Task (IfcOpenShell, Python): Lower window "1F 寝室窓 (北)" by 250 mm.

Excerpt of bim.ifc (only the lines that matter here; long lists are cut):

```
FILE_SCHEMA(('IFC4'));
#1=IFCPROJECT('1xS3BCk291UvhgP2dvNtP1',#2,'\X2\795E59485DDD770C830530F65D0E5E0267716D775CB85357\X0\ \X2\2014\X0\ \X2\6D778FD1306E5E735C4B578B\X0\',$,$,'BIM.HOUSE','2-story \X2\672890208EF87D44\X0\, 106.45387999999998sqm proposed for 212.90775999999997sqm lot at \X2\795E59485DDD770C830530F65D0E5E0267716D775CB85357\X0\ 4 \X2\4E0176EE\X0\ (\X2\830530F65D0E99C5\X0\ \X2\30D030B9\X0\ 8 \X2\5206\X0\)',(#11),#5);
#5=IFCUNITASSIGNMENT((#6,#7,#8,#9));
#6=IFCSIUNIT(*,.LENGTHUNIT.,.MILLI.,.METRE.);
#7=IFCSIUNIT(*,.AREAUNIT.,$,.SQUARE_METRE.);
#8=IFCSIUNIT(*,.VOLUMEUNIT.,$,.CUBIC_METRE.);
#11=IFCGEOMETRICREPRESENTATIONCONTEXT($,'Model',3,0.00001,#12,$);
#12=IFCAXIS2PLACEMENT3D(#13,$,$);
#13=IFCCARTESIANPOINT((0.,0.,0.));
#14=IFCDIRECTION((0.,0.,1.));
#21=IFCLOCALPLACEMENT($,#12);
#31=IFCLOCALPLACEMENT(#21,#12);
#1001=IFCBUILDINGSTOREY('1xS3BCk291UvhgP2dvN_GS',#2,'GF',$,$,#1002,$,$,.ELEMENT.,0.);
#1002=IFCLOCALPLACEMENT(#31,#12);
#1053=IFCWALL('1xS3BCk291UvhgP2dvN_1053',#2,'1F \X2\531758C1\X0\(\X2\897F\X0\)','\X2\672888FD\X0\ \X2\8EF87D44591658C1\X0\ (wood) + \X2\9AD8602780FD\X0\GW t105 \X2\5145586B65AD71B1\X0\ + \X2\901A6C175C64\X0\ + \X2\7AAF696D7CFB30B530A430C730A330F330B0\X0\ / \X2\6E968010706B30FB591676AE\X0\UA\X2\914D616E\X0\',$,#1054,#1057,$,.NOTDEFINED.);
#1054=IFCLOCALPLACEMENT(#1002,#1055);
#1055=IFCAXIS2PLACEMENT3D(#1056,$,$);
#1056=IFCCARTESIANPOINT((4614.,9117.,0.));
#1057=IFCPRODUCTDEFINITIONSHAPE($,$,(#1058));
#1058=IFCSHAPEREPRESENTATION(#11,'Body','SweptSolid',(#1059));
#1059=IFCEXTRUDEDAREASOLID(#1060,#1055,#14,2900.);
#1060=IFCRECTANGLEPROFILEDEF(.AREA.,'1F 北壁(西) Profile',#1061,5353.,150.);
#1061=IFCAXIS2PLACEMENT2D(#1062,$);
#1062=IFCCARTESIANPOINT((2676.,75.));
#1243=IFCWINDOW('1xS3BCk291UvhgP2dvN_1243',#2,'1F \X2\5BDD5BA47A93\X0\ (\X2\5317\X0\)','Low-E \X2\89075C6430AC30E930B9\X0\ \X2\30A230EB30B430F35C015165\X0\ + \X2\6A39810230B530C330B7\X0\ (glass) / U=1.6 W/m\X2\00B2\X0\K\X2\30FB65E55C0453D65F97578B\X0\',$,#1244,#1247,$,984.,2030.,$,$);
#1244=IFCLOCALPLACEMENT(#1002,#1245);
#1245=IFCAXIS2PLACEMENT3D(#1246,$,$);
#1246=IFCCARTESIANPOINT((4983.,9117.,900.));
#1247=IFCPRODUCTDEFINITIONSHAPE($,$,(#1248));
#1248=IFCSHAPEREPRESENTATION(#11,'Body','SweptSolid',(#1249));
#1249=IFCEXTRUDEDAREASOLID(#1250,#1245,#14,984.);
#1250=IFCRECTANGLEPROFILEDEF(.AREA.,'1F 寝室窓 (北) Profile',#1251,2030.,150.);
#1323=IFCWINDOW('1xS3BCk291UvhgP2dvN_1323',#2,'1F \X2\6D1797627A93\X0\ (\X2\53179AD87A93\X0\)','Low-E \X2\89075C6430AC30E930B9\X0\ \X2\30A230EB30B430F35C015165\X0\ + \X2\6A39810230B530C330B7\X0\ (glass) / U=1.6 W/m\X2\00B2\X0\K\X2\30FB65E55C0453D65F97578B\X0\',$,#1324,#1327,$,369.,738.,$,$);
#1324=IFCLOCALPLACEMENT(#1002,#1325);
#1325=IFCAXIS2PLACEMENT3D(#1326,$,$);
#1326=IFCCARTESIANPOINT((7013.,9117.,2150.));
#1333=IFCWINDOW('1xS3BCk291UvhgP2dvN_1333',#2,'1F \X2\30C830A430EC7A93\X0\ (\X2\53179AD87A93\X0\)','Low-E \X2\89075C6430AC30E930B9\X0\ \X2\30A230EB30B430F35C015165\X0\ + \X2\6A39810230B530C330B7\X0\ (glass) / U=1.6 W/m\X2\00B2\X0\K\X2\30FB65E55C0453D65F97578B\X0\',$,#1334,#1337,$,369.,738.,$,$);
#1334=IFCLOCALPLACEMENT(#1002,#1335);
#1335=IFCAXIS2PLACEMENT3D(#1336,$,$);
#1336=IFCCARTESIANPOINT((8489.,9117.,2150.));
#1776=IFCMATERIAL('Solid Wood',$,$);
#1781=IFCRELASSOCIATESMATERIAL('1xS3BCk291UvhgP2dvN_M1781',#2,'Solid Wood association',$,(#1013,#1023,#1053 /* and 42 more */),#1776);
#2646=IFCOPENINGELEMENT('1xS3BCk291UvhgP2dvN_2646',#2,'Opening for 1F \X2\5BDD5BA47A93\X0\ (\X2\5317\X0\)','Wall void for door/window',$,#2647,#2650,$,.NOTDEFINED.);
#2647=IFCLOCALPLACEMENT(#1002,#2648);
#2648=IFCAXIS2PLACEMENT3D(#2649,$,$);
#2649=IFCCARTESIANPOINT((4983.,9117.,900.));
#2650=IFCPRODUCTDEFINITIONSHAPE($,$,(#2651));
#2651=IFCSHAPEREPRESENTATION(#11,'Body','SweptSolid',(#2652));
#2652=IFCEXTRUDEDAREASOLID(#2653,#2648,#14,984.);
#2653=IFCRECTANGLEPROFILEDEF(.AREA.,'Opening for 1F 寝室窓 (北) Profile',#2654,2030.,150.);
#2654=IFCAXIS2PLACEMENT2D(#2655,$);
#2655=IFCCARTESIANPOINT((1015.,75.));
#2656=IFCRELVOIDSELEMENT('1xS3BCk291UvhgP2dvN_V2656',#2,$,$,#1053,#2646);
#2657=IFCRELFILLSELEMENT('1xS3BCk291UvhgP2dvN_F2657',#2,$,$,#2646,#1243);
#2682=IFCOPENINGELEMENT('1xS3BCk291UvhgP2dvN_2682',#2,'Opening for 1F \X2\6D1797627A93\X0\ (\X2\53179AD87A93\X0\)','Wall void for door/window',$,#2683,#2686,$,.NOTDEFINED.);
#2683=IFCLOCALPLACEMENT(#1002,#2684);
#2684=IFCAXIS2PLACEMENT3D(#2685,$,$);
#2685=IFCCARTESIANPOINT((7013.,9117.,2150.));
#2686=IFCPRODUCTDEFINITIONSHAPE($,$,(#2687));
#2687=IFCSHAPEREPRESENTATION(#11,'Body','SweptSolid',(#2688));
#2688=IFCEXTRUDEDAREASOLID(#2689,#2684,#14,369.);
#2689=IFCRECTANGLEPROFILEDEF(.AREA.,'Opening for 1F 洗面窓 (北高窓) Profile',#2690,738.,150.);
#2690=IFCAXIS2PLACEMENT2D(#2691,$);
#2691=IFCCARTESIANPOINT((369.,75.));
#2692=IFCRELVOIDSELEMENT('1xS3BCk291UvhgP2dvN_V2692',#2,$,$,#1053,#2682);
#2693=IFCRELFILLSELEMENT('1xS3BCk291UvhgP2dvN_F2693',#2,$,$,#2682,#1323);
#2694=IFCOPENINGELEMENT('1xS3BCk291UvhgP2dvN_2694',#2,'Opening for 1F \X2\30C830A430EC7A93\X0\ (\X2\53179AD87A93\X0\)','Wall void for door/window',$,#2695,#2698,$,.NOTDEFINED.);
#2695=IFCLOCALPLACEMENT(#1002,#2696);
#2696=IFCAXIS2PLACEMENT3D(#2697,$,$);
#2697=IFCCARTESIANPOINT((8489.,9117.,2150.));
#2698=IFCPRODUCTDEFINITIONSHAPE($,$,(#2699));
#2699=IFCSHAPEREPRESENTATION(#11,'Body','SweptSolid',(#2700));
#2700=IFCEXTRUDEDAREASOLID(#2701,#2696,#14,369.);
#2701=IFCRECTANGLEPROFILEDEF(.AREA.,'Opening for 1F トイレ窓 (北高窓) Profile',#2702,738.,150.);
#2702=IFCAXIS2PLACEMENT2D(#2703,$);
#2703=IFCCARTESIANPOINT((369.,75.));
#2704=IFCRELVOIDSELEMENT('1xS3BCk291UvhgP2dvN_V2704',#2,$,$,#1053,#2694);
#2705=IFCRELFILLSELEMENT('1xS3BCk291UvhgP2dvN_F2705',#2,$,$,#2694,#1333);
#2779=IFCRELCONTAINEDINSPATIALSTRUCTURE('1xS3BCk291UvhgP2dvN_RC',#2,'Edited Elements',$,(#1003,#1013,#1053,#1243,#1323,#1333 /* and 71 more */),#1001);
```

```python
import numpy as np
import ifcopenshell
import ifcopenshell.api.geometry
import ifcopenshell.util.placement
import ifcopenshell.util.unit

model = ifcopenshell.open("bim.ifc")
unit_scale = ifcopenshell.util.unit.calculate_unit_scale(model)

window = model.by_id(1243)
opening = window.FillsVoids[0].RelatingOpeningElement
dz = -0.25 / unit_scale

shift = np.array([0.0, 0.0, dz])
# The window is not placed relative to its opening, so move both.
for product in (opening, window):
    matrix = ifcopenshell.util.placement.get_local_placement(product.ObjectPlacement)
    matrix[:3, 3] += shift
    ifcopenshell.api.geometry.edit_object_placement(model, product=product, matrix=matrix, is_si=False)

print(f"moved by {dz * unit_scale:+.3f} m")

model.write("bim_updated.ifc")
```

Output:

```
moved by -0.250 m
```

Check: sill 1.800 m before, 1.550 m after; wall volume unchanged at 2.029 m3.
